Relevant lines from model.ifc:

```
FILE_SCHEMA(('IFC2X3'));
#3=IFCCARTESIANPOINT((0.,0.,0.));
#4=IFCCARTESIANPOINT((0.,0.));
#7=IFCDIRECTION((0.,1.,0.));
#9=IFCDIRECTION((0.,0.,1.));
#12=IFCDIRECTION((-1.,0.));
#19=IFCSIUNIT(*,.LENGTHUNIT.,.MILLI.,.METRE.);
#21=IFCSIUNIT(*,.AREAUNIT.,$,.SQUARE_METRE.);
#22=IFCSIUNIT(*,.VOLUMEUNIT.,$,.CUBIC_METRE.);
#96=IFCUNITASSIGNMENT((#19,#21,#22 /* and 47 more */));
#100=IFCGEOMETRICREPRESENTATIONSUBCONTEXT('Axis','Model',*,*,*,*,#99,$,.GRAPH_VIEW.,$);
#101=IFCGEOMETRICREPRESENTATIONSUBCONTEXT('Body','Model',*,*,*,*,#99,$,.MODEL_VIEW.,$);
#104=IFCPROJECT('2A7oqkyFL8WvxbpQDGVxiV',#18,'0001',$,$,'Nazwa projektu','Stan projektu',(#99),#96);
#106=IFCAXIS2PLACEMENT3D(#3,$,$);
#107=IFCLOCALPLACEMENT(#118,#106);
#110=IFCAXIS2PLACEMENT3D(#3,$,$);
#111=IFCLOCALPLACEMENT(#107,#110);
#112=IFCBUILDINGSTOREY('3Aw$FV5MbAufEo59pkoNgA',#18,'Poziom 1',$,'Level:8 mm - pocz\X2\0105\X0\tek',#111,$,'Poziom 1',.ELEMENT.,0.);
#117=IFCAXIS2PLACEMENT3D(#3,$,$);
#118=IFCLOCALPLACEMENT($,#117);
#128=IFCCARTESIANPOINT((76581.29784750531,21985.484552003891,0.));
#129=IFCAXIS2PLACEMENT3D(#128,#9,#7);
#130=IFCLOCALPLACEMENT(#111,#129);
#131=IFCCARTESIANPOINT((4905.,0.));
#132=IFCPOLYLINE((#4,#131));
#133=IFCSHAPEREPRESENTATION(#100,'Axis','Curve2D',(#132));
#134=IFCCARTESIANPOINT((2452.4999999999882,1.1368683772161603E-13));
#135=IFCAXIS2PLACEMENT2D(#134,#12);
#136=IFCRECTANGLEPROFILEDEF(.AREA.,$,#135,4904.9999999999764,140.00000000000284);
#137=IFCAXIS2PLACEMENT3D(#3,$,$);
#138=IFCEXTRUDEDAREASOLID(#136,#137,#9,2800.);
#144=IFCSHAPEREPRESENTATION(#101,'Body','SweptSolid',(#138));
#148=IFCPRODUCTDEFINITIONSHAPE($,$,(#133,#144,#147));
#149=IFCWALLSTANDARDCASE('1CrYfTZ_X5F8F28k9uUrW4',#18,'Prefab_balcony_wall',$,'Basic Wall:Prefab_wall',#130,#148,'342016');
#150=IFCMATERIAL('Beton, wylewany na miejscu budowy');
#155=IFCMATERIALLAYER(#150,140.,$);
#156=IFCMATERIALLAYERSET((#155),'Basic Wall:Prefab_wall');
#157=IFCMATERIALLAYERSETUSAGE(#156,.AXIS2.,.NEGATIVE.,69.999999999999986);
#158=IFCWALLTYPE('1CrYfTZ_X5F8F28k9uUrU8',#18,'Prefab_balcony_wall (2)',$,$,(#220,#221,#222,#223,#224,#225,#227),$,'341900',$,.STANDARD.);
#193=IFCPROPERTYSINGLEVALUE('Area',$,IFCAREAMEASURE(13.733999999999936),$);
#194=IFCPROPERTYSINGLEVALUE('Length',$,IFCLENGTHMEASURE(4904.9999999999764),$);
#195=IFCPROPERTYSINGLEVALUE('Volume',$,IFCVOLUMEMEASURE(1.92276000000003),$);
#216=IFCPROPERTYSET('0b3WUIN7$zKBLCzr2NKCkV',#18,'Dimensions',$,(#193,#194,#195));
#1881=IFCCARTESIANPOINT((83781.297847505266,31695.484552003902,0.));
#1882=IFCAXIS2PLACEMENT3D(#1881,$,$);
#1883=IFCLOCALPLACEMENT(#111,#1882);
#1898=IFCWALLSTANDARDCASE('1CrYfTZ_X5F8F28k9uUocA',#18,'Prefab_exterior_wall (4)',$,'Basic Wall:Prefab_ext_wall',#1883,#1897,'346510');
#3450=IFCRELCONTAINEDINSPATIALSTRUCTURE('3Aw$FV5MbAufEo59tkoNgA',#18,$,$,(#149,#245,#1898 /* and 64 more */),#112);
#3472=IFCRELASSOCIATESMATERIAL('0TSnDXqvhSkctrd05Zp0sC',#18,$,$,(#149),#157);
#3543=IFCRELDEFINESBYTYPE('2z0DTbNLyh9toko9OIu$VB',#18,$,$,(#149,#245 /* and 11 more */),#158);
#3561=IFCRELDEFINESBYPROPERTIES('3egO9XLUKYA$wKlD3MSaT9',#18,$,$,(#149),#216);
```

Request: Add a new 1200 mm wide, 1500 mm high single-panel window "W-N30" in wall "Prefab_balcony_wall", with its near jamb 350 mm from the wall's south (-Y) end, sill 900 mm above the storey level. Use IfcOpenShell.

```python
import numpy as np
import ifcopenshell
import ifcopenshell.api.feature
import ifcopenshell.api.geometry
import ifcopenshell.api.pset
import ifcopenshell.api.root
import ifcopenshell.api.spatial
import ifcopenshell.api.type
import ifcopenshell.geom
import ifcopenshell.util.element
import ifcopenshell.util.placement
import ifcopenshell.util.representation
import ifcopenshell.util.shape
import ifcopenshell.util.unit

model = ifcopenshell.open("model.ifc")
unit_scale = ifcopenshell.util.unit.calculate_unit_scale(model)
area_scale = ifcopenshell.util.unit.calculate_unit_scale(model, "AREAUNIT")
volume_scale = ifcopenshell.util.unit.calculate_unit_scale(model, "VOLUMEUNIT")
settings = ifcopenshell.geom.settings()


def volume(element):
    """Net volume in cubic metres, openings subtracted."""
    shape = ifcopenshell.geom.create_shape(settings, element)
    return ifcopenshell.util.shape.get_volume(shape.geometry)


wall = model.by_guid("1CrYfTZ_X5F8F28k9uUrW4")
storey = ifcopenshell.util.element.get_container(wall, ifc_class="IfcBuildingStorey")
context = ifcopenshell.util.representation.get_context(model, "Model", "Body", "MODEL_VIEW")
before = volume(wall)

width, height, from_end, sill = 1.2, 1.5, 0.35, 0.9  # metres

# The wall runs along its own X axis, and the end named is its -X end.
wall_shape = ifcopenshell.geom.create_shape(settings, wall)
x, y, z = ifcopenshell.util.shape.get_vertices(wall_shape.geometry).T
start = x.min() + from_end
face, thickness = float(y.min()), float(y.max() - y.min())
wall_matrix = ifcopenshell.util.placement.get_local_placement(wall.ObjectPlacement)
level = ifcopenshell.util.placement.get_local_placement(storey.ObjectPlacement)[2, 3]


def in_wall(x, y):
    """Placement at x, y metres in the wall's axes, at sill height."""
    matrix = wall_matrix.copy()
    matrix[:, 3] = wall_matrix @ np.array([x / unit_scale, y / unit_scale, 0.0, 1.0])
    matrix[2, 3] = level + sill / unit_scale
    return matrix


# Opening: a box that overshoots both wall faces by 50 mm.
opening = ifcopenshell.api.root.create_entity(model, ifc_class="IfcOpeningElement")
box = ifcopenshell.api.geometry.add_wall_representation(
    model, context=context, length=width, height=height, thickness=thickness + 0.1
)
ifcopenshell.api.geometry.assign_representation(model, product=opening, representation=box)
ifcopenshell.api.geometry.edit_object_placement(model, product=opening, matrix=in_wall(start, face - 0.05), is_si=False)
ifcopenshell.api.feature.add_feature(model, feature=opening, element=wall)

window = ifcopenshell.api.root.create_entity(model, ifc_class="IfcWindow", name="W-N30")
window.OverallWidth, window.OverallHeight = width / unit_scale, height / unit_scale
body = ifcopenshell.api.geometry.add_window_representation(
    model,
    context=context,
    overall_width=window.OverallWidth,
    overall_height=window.OverallHeight,
    partition_type="SINGLE_PANEL",
)
ifcopenshell.api.geometry.assign_representation(model, product=window, representation=body)
ifcopenshell.api.spatial.assign_container(model, products=[window], relating_structure=storey)
fills = ifcopenshell.api.feature.add_filling(model, opening=opening, element=window)
fills.OwnerHistory = window.OwnerHistory  # required in IFC2X3

# IFC2X3 keeps the operation on the window style.
style = ifcopenshell.api.root.create_entity(model, ifc_class="IfcWindowStyle", name="W-N30")
style.OperationType, style.ConstructionType = "SINGLE_PANEL", "NOTDEFINED"
style.ParameterTakesPrecedence = style.Sizeable = False
ifcopenshell.api.type.assign_type(model, related_objects=[window], relating_type=style)

# Centre the window in the wall's thickness.
ifcopenshell.api.geometry.edit_object_placement(model, product=window, matrix=in_wall(start, face), is_si=False)
window_shape = ifcopenshell.geom.create_shape(settings, window)
depth = ifcopenshell.util.shape.get_vertices(window_shape.geometry)[:, 1]
offset = face + thickness / 2 - (depth.min() + depth.max()) / 2
ifcopenshell.api.geometry.edit_object_placement(model, product=window, matrix=in_wall(start, offset), is_si=False)

after = volume(wall)

# Update the wall's stored quantities.
pset = model.by_id(ifcopenshell.util.element.get_pset(wall, "Dimensions", should_inherit=False)["id"])
ifcopenshell.api.pset.edit_pset(model, pset=pset, properties={
    "Area": model.create_entity("IfcAreaMeasure", after / thickness / area_scale),
    "Volume": model.create_entity("IfcVolumeMeasure", after / volume_scale),
})

print(f"wall volume {before:.3f} -> {after:.3f} m3")

model.write("model_updated.ifc")
```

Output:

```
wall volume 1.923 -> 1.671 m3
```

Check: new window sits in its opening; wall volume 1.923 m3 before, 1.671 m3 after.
